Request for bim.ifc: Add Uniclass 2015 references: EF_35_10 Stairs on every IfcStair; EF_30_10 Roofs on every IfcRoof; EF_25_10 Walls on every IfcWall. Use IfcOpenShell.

First a look at what the model holds.

```python
import ifcopenshell

model = ifcopenshell.open("bim.ifc")
print(model.schema)
print("classifications:", [c.Name for c in model.by_type("IfcClassification")])
for ifc_class in ("IfcDoor", "IfcRoof", "IfcStair", "IfcWall", "IfcWindow"):
    print(ifc_class, len(model.by_type(ifc_class)))
```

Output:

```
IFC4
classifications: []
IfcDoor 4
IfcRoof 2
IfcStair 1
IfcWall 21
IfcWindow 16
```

```python
import ifcopenshell
import ifcopenshell.api.classification

model = ifcopenshell.open("bim.ifc")

system = ifcopenshell.api.classification.add_classification(model, classification="Uniclass 2015")

codes = {
    "IfcStair": ("EF_35_10", "Stairs"),
    "IfcRoof": ("EF_30_10", "Roofs"),
    "IfcWall": ("EF_25_10", "Walls"),
}
for ifc_class, (code, name) in codes.items():
    products = model.by_type(ifc_class)
    ifcopenshell.api.classification.add_reference(
        model, products=products, classification=system, identification=code, name=name
    )
    print(code, len(products))

model.write("bim_edited.ifc")
```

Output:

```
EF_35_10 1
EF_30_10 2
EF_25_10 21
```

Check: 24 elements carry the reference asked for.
